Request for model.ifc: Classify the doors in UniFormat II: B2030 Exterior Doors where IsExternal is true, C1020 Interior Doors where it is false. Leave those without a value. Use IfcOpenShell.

First a look at what the model holds.

```python
import ifcopenshell
import ifcopenshell.util.element

model = ifcopenshell.open("model.ifc")
print(model.schema)
print("classifications:", [c.Name for c in model.by_type("IfcClassification")])
values = [ifcopenshell.util.element.get_pset(e, "Pset_DoorCommon", "IsExternal") for e in model.by_type("IfcDoor")]
for value in (True, False, None):
    print("IsExternal", value, values.count(value))
```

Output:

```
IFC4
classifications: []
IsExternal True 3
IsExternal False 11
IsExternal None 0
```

```python
import ifcopenshell
import ifcopenshell.api.classification
import ifcopenshell.util.element

model = ifcopenshell.open("model.ifc")

system = ifcopenshell.api.classification.add_classification(model, classification="UniFormat II")

doors = model.by_type("IfcDoor")
external = {e: ifcopenshell.util.element.get_pset(e, "Pset_DoorCommon", "IsExternal") for e in doors}
for flag, code, name in ((True, "B2030", "Exterior Doors"), (False, "C1020", "Interior Doors")):
    products = [e for e in doors if external[e] is flag]
    ifcopenshell.api.classification.add_reference(
        model, products=products, classification=system, identification=code, name=name
    )
    print(code, len(products))

model.write("model_v2.ifc")
```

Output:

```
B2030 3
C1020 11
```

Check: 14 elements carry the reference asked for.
